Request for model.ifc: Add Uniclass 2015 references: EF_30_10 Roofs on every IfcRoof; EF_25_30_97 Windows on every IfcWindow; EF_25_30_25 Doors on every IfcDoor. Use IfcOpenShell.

First a look at what the model holds.

```python
import ifcopenshell

model = ifcopenshell.open("model.ifc")
print(model.schema)
print("classifications:", [c.Name for c in model.by_type("IfcClassification")])
for ifc_class in ("IfcDoor", "IfcRoof", "IfcStair", "IfcWall", "IfcWindow"):
    print(ifc_class, len(model.by_type(ifc_class)))
```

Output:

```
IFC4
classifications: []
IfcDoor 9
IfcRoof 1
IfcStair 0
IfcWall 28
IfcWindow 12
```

```python
import ifcopenshell
import ifcopenshell.api.classification

model = ifcopenshell.open("model.ifc")

system = ifcopenshell.api.classification.add_classification(model, classification="Uniclass 2015")

codes = {
    "IfcRoof": ("EF_30_10", "Roofs"),
    "IfcWindow": ("EF_25_30_97", "Windows"),
    "IfcDoor": ("EF_25_30_25", "Doors"),
}
for ifc_class, (code, name) in codes.items():
    products = model.by_type(ifc_class)
    ifcopenshell.api.classification.add_reference(
        model, products=products, classification=system, identification=code, name=name
    )
    print(code, len(products))

model.write("model_rev.ifc")
```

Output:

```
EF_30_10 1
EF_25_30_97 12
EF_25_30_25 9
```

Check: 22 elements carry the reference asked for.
